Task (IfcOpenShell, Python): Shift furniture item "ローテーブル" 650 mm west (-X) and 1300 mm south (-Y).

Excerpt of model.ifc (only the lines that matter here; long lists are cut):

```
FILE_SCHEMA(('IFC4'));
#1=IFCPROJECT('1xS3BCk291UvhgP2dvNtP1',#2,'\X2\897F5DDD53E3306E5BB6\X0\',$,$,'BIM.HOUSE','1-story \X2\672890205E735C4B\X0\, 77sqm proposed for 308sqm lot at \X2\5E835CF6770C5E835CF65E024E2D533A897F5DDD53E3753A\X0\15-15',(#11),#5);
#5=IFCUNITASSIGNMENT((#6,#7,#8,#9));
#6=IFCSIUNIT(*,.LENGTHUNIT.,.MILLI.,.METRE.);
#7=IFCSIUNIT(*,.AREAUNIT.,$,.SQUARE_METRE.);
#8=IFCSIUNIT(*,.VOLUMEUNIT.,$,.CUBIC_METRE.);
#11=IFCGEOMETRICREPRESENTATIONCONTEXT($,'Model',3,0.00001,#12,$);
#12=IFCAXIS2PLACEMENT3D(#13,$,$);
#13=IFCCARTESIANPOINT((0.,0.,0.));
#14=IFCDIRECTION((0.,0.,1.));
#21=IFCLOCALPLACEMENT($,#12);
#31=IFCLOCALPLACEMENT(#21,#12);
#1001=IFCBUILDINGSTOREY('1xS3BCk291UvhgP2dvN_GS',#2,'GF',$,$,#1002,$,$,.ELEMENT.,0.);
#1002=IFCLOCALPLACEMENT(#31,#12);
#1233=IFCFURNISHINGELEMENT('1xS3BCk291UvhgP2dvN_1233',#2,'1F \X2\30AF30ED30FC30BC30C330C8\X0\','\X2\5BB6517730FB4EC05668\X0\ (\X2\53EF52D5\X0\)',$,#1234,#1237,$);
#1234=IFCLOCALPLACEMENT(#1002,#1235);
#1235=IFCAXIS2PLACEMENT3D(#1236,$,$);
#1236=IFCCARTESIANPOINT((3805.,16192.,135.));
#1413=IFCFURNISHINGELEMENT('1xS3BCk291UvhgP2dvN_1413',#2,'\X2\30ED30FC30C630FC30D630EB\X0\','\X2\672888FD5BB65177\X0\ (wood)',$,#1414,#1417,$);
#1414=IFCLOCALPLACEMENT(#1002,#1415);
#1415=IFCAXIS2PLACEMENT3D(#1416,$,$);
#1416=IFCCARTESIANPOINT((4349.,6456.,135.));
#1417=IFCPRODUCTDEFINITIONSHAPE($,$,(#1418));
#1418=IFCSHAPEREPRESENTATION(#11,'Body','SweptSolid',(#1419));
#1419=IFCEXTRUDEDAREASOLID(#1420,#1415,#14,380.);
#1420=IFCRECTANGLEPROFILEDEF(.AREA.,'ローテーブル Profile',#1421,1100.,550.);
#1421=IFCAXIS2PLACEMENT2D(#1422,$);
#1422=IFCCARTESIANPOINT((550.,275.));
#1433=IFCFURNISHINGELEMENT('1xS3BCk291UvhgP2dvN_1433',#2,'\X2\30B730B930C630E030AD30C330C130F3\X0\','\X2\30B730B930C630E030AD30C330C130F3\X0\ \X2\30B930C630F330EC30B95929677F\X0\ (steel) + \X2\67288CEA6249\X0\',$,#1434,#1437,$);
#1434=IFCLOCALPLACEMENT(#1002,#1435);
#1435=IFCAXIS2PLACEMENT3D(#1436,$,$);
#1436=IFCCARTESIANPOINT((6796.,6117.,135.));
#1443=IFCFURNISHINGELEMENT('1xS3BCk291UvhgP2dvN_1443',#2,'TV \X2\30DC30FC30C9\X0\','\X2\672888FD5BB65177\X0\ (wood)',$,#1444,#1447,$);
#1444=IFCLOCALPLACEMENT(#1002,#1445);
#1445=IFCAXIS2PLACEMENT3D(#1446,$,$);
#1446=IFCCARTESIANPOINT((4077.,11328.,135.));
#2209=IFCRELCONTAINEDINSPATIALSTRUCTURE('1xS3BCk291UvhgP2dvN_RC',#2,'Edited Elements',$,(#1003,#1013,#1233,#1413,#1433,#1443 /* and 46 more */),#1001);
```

```python
import ifcopenshell
import ifcopenshell.api.geometry
import ifcopenshell.util.placement
import ifcopenshell.util.unit

model = ifcopenshell.open("model.ifc")
unit_scale = ifcopenshell.util.unit.calculate_unit_scale(model)

item = model.by_guid("1xS3BCk291UvhgP2dvN_1413")
matrix = ifcopenshell.util.placement.get_local_placement(item.ObjectPlacement)
matrix[0, 3] -= 0.65 / unit_scale
matrix[1, 3] -= 1.3 / unit_scale
ifcopenshell.api.geometry.edit_object_placement(model, product=item, matrix=matrix, is_si=False)

print(ifcopenshell.util.placement.get_local_placement(item.ObjectPlacement).round(3) + 0.0)

model.write("model_rev.ifc")
```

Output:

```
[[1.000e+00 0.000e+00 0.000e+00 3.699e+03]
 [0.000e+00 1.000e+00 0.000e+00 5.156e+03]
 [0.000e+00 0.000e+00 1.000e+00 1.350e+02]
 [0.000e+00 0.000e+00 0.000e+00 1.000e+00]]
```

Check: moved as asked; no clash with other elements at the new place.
